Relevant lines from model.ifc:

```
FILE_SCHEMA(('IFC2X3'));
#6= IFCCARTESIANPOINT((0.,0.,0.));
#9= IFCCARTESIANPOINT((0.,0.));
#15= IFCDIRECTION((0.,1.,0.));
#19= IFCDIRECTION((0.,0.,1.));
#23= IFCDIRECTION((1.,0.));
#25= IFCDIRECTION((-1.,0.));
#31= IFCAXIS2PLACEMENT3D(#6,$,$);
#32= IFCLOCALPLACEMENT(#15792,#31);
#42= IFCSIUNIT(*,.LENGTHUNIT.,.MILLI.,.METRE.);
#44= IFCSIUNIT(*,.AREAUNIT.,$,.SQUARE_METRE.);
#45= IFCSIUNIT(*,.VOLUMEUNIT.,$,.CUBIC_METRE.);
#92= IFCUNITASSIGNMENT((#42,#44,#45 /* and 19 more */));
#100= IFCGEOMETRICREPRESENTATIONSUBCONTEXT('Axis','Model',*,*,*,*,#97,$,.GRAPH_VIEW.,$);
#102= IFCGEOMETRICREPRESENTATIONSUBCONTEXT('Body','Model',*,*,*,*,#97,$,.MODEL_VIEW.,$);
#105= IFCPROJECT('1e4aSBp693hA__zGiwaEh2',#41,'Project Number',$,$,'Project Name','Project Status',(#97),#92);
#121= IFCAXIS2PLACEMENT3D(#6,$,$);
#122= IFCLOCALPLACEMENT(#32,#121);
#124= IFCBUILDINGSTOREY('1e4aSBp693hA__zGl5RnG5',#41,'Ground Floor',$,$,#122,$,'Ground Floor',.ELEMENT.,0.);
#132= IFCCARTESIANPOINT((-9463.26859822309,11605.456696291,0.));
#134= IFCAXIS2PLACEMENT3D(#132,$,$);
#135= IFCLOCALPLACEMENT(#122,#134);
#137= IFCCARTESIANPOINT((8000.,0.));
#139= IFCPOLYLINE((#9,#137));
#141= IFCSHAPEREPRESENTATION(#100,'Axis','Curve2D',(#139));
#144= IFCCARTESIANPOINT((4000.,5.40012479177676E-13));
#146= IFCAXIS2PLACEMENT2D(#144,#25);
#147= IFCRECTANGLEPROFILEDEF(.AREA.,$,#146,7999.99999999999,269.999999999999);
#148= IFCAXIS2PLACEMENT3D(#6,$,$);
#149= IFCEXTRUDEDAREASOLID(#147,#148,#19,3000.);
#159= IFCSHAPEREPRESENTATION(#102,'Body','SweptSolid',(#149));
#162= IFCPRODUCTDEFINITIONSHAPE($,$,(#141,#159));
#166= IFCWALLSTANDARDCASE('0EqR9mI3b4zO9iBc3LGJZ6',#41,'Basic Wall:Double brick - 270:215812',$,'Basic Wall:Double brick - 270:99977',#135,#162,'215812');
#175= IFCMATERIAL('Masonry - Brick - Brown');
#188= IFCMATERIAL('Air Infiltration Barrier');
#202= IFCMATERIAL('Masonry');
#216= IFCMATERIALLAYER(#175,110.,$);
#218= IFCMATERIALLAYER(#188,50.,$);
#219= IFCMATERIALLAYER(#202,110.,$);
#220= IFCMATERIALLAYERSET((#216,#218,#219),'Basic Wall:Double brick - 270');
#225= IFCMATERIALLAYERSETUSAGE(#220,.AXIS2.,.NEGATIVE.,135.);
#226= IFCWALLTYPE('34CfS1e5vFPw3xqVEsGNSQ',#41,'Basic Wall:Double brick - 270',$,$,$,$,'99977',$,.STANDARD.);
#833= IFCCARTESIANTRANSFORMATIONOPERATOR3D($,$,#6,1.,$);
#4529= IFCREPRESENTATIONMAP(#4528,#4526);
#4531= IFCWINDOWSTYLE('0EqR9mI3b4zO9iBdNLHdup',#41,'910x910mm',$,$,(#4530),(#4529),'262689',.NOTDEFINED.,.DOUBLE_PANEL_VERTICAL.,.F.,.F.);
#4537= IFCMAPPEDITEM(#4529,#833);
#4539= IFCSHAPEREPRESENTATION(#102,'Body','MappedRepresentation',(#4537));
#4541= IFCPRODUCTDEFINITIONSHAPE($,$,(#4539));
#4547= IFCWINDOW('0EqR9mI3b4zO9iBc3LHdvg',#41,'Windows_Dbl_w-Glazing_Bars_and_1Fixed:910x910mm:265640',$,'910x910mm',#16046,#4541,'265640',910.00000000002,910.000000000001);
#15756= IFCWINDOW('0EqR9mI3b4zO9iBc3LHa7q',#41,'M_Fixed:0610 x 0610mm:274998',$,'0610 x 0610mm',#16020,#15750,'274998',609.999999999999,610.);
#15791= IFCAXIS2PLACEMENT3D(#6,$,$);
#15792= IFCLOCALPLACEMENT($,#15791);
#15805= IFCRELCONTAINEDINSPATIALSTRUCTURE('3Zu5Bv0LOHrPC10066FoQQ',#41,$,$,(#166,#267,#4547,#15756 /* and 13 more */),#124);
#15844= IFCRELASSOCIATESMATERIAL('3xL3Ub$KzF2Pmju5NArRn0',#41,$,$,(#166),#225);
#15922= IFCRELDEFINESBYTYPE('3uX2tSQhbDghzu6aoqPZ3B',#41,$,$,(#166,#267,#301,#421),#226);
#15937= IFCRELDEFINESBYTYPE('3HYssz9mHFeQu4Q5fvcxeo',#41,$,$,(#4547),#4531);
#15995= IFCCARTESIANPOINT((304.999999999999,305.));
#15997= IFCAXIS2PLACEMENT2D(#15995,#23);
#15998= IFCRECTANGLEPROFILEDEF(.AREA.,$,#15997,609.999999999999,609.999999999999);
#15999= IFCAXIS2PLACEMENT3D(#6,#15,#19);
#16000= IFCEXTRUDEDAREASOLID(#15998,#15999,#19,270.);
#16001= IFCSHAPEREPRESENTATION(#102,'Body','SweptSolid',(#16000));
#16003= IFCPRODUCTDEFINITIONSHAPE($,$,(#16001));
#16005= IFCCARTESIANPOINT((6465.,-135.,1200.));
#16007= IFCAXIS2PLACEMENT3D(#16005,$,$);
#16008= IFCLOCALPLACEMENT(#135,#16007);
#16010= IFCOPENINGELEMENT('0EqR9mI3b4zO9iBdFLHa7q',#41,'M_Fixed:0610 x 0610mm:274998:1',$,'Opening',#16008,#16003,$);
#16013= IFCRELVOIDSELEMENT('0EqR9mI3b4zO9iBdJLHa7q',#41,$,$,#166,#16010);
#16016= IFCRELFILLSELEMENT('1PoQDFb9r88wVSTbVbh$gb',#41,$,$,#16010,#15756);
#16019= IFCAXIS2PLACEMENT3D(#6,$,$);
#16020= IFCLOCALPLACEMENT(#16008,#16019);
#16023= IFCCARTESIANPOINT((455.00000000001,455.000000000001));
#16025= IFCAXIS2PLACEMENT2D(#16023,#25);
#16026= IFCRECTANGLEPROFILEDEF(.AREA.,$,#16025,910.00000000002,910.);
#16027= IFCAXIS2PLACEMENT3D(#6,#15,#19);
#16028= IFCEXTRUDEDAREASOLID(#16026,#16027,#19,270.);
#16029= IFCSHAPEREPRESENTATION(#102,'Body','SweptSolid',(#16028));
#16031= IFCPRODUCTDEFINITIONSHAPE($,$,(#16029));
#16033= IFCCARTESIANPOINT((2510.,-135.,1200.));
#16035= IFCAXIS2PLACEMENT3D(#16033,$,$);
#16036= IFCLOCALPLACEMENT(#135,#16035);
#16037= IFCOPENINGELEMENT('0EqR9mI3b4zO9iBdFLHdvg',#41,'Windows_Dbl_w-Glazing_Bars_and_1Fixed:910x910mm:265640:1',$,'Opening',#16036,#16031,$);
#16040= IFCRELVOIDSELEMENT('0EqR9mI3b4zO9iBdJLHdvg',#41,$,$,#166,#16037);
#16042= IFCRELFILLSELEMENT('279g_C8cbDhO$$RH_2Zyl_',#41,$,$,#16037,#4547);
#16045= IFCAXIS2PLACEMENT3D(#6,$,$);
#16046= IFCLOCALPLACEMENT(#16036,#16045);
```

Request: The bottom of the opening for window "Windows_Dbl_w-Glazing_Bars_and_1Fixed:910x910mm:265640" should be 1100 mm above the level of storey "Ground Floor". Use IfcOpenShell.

```python
import numpy as np
import ifcopenshell
import ifcopenshell.api.geometry
import ifcopenshell.geom
import ifcopenshell.util.element
import ifcopenshell.util.placement
import ifcopenshell.util.shape
import ifcopenshell.util.unit

model = ifcopenshell.open("model.ifc")
unit_scale = ifcopenshell.util.unit.calculate_unit_scale(model)

window = model.by_id(4547)
opening = window.FillsVoids[0].RelatingOpeningElement
storey = ifcopenshell.util.element.get_container(window, ifc_class="IfcBuildingStorey")
level = ifcopenshell.util.placement.get_local_placement(storey.ObjectPlacement)[2, 3]

# The opening's origin need not be at the sill, so measure its lowest point.
shape = ifcopenshell.geom.create_shape(ifcopenshell.geom.settings(), opening)
bottom = ifcopenshell.util.shape.get_shape_bottom_elevation(shape, shape.geometry) / unit_scale
dz = level + 1100.0 - bottom

shift = np.array([0.0, 0.0, dz])
# The window is placed relative to its opening, so it follows when the opening moves.
matrix = ifcopenshell.util.placement.get_local_placement(opening.ObjectPlacement)
matrix[:3, 3] += shift
ifcopenshell.api.geometry.edit_object_placement(
    model, product=opening, matrix=matrix, is_si=False, should_transform_children=True
)

print(f"moved by {dz * unit_scale:+.3f} m")

model.write("model-out.ifc")
```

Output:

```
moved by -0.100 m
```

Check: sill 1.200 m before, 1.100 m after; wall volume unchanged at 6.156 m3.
